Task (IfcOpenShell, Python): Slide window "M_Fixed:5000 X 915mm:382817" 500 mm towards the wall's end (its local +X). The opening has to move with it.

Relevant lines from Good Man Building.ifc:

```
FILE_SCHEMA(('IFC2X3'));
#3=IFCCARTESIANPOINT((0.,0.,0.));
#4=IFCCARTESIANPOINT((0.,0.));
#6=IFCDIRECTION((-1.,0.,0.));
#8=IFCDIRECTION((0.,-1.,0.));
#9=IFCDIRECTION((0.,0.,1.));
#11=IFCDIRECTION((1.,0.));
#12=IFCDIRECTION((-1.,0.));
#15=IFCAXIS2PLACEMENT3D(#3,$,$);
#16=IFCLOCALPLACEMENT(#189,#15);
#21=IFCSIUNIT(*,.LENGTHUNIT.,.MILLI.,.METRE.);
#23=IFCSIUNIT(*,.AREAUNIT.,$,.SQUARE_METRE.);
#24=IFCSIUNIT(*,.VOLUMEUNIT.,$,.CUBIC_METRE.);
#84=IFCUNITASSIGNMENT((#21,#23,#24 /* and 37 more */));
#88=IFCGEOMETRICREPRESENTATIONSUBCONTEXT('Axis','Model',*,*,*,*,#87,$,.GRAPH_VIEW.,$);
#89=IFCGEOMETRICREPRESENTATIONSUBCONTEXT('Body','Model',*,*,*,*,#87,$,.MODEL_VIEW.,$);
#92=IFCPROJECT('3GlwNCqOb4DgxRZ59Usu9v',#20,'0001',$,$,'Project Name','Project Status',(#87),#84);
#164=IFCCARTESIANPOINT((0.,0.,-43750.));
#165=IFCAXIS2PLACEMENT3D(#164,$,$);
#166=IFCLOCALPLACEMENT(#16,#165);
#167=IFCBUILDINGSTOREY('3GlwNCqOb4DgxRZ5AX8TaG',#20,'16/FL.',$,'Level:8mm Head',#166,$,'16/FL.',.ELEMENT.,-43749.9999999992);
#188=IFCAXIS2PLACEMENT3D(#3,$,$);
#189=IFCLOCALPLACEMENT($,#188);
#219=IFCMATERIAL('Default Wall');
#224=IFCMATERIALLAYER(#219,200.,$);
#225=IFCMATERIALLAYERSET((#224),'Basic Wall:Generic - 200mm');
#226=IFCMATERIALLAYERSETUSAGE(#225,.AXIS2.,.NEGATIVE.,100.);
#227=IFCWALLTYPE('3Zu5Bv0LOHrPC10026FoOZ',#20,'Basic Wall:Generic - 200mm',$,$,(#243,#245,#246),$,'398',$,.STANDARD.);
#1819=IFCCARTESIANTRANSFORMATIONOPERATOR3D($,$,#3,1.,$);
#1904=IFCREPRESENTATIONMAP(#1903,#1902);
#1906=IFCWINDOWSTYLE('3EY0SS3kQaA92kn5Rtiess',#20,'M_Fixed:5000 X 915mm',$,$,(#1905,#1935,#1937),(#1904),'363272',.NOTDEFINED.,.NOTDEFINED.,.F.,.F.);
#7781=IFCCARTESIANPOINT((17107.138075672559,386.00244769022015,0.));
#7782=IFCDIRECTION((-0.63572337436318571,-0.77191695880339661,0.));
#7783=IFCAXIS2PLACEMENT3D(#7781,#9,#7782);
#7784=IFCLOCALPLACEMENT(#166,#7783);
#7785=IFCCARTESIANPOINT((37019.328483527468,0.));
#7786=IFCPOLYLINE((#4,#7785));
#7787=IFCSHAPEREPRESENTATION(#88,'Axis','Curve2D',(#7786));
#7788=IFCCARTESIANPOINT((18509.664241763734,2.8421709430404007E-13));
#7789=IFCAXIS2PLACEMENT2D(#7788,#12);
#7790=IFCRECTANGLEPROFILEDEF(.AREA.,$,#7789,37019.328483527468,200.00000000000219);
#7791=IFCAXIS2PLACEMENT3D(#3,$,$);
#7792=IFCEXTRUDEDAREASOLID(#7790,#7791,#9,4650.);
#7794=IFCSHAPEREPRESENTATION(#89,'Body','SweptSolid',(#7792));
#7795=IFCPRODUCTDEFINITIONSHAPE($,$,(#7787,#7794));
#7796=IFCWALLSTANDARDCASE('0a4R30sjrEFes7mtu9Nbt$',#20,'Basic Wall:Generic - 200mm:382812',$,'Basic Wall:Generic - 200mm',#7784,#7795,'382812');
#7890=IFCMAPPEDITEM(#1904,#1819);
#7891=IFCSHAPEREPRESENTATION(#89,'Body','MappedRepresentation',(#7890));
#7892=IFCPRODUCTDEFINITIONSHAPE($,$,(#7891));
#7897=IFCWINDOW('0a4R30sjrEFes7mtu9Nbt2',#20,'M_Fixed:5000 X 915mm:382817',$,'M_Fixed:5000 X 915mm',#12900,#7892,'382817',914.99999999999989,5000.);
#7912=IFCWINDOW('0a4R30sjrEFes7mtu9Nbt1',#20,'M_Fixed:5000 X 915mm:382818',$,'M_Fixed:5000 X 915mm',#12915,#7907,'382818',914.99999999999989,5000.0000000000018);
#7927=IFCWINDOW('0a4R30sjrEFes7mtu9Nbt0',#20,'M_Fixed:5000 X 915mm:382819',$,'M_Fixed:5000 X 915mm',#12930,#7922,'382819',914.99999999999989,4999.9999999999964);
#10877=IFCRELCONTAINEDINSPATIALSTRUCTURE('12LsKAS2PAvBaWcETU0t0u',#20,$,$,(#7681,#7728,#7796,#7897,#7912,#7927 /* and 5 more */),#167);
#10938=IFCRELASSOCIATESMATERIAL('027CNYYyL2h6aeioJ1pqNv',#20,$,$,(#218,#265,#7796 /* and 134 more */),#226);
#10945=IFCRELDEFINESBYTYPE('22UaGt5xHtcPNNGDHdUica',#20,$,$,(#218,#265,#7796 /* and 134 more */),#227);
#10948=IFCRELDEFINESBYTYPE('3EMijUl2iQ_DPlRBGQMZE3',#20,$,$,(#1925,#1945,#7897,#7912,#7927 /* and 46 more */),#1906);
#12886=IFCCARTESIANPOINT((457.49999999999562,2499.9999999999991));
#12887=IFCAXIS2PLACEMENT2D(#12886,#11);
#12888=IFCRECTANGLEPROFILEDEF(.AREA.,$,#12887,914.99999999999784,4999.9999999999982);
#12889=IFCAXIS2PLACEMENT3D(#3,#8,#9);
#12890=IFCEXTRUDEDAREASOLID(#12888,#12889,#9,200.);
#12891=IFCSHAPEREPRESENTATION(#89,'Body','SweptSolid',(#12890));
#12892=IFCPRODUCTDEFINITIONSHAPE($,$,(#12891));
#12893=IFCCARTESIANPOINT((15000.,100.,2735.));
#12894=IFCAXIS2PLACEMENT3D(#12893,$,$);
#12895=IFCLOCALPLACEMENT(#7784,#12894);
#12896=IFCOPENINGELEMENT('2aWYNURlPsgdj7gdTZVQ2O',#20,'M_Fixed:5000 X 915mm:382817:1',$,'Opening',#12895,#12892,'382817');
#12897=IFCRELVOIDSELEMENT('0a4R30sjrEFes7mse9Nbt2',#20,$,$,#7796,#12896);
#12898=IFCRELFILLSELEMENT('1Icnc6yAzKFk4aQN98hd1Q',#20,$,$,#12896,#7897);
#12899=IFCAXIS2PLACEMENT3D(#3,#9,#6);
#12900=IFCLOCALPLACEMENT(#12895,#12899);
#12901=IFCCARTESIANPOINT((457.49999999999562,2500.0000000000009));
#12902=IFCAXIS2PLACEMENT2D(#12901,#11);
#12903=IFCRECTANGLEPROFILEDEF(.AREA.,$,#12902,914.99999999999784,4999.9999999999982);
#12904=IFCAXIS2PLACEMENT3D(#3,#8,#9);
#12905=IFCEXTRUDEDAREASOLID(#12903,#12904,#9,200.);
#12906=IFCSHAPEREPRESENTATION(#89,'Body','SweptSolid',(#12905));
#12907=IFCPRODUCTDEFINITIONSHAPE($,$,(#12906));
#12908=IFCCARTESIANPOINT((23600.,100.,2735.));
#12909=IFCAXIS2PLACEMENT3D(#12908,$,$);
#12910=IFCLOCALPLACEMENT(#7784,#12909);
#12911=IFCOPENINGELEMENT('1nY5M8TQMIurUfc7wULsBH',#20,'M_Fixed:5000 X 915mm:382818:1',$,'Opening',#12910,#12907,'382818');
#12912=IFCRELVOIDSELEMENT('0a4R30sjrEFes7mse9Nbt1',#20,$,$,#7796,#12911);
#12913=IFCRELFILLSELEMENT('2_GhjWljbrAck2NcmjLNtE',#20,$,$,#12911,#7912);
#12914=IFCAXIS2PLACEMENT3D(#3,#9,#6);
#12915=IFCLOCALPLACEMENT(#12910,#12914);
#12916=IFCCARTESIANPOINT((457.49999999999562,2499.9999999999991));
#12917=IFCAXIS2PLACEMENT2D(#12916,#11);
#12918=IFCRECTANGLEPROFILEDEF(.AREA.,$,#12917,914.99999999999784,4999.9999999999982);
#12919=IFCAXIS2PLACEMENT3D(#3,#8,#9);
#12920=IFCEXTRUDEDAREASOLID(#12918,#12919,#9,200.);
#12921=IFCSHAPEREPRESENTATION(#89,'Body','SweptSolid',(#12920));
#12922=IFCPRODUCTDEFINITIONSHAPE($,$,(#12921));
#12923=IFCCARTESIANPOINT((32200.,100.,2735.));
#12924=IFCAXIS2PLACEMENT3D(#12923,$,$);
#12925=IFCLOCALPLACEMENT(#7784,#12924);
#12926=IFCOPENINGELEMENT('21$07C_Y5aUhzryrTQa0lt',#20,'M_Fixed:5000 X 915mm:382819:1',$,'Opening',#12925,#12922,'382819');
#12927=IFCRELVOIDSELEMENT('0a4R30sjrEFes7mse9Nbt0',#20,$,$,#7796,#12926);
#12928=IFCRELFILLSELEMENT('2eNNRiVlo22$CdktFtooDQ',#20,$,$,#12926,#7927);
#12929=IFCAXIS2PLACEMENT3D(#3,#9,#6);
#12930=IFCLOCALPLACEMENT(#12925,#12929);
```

```python
import ifcopenshell
import ifcopenshell.api.geometry
import ifcopenshell.util.placement

model = ifcopenshell.open("Good Man Building.ifc")

window = model.by_guid("0a4R30sjrEFes7mtu9Nbt2")
opening = window.FillsVoids[0].RelatingOpeningElement
wall = opening.VoidsElements[0].RelatingBuildingElement

wall_matrix = ifcopenshell.util.placement.get_local_placement(wall.ObjectPlacement)
shift = wall_matrix[:3, 0] * 500.0
before = ifcopenshell.util.placement.get_local_placement(window.ObjectPlacement)[:3, 3].copy()

# The window is placed relative to its opening, so it follows when the opening moves.
matrix = ifcopenshell.util.placement.get_local_placement(opening.ObjectPlacement)
matrix[:3, 3] += shift
ifcopenshell.api.geometry.edit_object_placement(
    model, product=opening, matrix=matrix, is_si=False, should_transform_children=True
)

after = ifcopenshell.util.placement.get_local_placement(window.ObjectPlacement)[:3, 3]
print("window moved by", (after - before).round(3) + 0.0)

model.write("Good Man Building_edited.ifc")
```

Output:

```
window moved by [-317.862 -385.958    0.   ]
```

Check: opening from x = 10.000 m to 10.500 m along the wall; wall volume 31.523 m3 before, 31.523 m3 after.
